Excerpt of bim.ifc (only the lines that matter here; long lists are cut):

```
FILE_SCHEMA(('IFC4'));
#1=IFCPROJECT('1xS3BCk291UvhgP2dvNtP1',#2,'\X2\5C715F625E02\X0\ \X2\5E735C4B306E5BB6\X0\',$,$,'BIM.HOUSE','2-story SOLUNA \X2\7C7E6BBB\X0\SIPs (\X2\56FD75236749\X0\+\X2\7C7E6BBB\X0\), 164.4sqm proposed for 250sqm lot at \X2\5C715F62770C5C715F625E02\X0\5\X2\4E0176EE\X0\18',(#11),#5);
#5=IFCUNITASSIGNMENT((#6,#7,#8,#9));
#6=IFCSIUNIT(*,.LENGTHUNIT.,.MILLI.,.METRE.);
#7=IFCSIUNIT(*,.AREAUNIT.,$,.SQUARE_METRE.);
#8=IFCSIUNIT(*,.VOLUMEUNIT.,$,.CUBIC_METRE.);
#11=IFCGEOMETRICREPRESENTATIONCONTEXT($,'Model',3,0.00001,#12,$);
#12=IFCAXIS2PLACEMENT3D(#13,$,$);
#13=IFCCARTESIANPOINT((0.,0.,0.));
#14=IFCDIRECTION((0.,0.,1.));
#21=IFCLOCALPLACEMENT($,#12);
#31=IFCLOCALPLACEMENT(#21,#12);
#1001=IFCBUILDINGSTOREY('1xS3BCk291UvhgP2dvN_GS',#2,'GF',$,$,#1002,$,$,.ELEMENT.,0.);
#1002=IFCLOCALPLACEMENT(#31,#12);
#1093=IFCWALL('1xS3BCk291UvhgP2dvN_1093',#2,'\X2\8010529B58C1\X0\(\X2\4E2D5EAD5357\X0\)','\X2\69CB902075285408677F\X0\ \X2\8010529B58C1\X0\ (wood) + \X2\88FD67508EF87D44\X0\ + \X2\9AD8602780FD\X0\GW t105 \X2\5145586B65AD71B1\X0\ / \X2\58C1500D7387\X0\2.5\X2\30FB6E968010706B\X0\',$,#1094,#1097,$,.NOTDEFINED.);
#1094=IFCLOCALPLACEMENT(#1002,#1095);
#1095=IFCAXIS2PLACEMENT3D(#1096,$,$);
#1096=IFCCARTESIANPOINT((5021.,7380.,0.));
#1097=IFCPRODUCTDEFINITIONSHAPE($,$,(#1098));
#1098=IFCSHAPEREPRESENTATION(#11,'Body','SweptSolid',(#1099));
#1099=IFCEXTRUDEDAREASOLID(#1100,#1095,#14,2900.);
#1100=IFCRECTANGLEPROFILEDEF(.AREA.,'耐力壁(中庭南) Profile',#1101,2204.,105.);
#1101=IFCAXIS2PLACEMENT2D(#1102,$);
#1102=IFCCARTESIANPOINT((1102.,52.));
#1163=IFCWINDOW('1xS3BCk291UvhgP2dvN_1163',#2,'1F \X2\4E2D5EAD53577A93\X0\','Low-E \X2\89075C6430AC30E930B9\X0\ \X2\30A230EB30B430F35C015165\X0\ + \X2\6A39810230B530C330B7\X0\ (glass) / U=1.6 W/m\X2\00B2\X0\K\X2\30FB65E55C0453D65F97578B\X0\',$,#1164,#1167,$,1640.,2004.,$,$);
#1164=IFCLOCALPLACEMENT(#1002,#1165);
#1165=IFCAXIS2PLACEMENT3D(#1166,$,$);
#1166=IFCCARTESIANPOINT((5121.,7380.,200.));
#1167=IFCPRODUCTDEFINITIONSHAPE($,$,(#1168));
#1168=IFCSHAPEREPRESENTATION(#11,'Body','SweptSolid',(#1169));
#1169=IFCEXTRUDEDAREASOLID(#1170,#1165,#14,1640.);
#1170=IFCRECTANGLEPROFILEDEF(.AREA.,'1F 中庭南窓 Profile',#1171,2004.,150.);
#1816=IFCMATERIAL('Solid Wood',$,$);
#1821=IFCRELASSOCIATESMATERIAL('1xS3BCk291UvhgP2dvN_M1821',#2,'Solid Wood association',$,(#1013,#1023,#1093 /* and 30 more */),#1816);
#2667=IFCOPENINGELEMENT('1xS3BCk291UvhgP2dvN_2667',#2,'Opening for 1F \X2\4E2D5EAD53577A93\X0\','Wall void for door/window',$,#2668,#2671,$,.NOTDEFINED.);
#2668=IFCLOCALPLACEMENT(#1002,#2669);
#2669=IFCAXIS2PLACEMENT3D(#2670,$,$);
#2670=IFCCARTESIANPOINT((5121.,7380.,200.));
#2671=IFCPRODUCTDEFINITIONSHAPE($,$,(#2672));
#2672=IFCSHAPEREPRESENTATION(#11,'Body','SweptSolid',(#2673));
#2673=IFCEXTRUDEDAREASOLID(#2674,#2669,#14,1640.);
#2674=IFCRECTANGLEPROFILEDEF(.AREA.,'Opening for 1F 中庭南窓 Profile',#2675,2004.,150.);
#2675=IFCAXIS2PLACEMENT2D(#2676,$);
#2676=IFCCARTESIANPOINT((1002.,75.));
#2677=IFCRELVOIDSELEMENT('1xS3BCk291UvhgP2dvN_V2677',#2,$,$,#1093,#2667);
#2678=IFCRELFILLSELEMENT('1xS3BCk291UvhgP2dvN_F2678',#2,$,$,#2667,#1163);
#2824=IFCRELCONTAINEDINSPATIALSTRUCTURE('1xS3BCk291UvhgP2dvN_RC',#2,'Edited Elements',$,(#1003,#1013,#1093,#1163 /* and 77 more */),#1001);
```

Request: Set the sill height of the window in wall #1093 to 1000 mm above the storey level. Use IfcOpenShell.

```python
import numpy as np
import ifcopenshell
import ifcopenshell.api.geometry
import ifcopenshell.geom
import ifcopenshell.util.element
import ifcopenshell.util.placement
import ifcopenshell.util.shape
import ifcopenshell.util.unit

model = ifcopenshell.open("bim.ifc")
unit_scale = ifcopenshell.util.unit.calculate_unit_scale(model)

window = model.by_id(1163)
opening = window.FillsVoids[0].RelatingOpeningElement
storey = ifcopenshell.util.element.get_container(window, ifc_class="IfcBuildingStorey")
level = ifcopenshell.util.placement.get_local_placement(storey.ObjectPlacement)[2, 3]

# The opening's origin need not be at the sill, so measure its lowest point.
shape = ifcopenshell.geom.create_shape(ifcopenshell.geom.settings(), opening)
bottom = ifcopenshell.util.shape.get_shape_bottom_elevation(shape, shape.geometry) / unit_scale
dz = level + 1 / unit_scale - bottom

shift = np.array([0.0, 0.0, dz])
# The window is not placed relative to its opening, so move both.
for product in (opening, window):
    matrix = ifcopenshell.util.placement.get_local_placement(product.ObjectPlacement)
    matrix[:3, 3] += shift
    ifcopenshell.api.geometry.edit_object_placement(model, product=product, matrix=matrix, is_si=False)

print(f"moved by {dz * unit_scale:+.3f} m")

model.write("bim_edited.ifc")
```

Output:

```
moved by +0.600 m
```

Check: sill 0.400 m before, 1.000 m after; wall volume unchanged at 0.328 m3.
